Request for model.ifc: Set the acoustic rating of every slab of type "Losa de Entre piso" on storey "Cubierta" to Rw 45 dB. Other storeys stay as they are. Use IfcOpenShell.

First a look at what the model holds.

```python
import ifcopenshell
import ifcopenshell.util.element

model = ifcopenshell.open("model.ifc")
print(model.schema)
storey = next(s for s in model.by_type("IfcBuildingStorey") if s.Name == "Cubierta")
slabs = [e for e in ifcopenshell.util.element.get_decomposition(storey) if e.is_a("IfcSlab")]
seen = {}
for e in slabs:
    element_type = ifcopenshell.util.element.get_type(e)
    key = (element_type.Name if element_type != e and element_type else None, ifcopenshell.util.element.get_pset(e, "Pset_SlabCommon", "AcousticRating"))
    seen[key] = seen.get(key, 0) + 1
for (name, value), count in sorted(seen.items(), key=str):
    print(count, "x", name, "|", value)
```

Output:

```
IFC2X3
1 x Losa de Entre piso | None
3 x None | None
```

```python
import ifcopenshell
import ifcopenshell.api.pset
import ifcopenshell.util.element

model = ifcopenshell.open("model.ifc")

storey = next(s for s in model.by_type("IfcBuildingStorey") if s.Name == "Cubierta")
slabs = [e for e in ifcopenshell.util.element.get_decomposition(storey) if e.is_a("IfcSlab")]

count = 0
for e in slabs:
    element_type = ifcopenshell.util.element.get_type(e)
    if element_type in (None, e) or element_type.Name != "Losa de Entre piso":
        continue
    # add_pset returns the element's existing set when there is one.
    pset = ifcopenshell.api.pset.add_pset(model, product=e, name="Pset_SlabCommon")
    ifcopenshell.api.pset.edit_pset(model, pset=pset, properties={"AcousticRating": "Rw 45 dB"})
    count += 1

print(count, "slabs updated")

model.write("model_updated.ifc")
```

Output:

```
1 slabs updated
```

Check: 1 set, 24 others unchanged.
